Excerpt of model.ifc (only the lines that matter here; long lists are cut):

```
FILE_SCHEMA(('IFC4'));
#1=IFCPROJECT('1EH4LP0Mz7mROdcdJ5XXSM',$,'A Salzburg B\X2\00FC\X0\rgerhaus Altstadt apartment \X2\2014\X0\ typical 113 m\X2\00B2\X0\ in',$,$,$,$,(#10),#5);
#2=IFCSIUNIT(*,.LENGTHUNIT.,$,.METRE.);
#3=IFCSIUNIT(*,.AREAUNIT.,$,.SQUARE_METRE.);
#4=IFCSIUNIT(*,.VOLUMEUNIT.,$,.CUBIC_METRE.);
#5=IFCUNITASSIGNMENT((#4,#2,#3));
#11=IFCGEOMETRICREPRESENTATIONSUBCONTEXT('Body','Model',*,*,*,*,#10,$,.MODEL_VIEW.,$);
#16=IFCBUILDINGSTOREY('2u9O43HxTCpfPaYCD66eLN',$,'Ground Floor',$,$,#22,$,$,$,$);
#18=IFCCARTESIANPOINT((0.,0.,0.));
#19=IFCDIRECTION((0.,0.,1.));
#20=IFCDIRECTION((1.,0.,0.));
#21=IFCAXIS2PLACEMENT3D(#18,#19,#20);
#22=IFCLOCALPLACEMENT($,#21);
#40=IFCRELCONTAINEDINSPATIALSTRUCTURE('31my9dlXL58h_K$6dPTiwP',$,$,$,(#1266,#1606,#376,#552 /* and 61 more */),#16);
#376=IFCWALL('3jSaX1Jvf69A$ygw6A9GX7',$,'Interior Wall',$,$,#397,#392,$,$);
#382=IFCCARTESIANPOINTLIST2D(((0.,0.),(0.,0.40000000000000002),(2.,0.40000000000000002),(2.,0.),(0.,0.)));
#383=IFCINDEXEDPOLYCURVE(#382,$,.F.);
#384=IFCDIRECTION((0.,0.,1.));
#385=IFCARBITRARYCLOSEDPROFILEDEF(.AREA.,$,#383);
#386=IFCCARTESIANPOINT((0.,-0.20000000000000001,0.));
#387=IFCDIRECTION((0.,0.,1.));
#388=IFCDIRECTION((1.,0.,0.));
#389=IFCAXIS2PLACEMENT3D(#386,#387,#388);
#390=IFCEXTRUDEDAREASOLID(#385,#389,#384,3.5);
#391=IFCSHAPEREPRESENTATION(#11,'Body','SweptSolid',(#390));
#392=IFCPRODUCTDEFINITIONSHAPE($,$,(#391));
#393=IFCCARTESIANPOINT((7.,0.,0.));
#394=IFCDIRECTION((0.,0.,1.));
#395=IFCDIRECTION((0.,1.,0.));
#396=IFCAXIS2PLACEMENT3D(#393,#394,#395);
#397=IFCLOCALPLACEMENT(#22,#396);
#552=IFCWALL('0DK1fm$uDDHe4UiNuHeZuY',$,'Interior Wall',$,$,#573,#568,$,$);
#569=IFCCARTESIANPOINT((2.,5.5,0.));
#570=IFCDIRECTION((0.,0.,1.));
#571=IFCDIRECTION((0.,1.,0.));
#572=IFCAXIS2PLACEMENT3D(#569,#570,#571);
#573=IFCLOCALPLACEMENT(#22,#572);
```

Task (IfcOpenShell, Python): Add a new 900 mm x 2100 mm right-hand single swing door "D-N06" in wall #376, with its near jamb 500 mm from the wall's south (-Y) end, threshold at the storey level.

```python
import numpy as np
import ifcopenshell
import ifcopenshell.api.feature
import ifcopenshell.api.geometry
import ifcopenshell.api.root
import ifcopenshell.api.spatial
import ifcopenshell.geom
import ifcopenshell.util.element
import ifcopenshell.util.placement
import ifcopenshell.util.representation
import ifcopenshell.util.shape
import ifcopenshell.util.unit

model = ifcopenshell.open("model.ifc")
unit_scale = ifcopenshell.util.unit.calculate_unit_scale(model)
settings = ifcopenshell.geom.settings()


def volume(element):
    """Net volume in cubic metres, openings subtracted."""
    shape = ifcopenshell.geom.create_shape(settings, element)
    return ifcopenshell.util.shape.get_volume(shape.geometry)


wall = model.by_id(376)
storey = ifcopenshell.util.element.get_container(wall, ifc_class="IfcBuildingStorey")
context = ifcopenshell.util.representation.get_context(model, "Model", "Body", "MODEL_VIEW")
before = volume(wall)

width, height, from_end, sill = 0.9, 2.1, 0.5, 0.0  # metres

# The wall runs along its own X axis, and the end named is its -X end.
wall_shape = ifcopenshell.geom.create_shape(settings, wall)
x, y, z = ifcopenshell.util.shape.get_vertices(wall_shape.geometry).T
start = x.min() + from_end
face, thickness = float(y.min()), float(y.max() - y.min())
wall_matrix = ifcopenshell.util.placement.get_local_placement(wall.ObjectPlacement)
level = ifcopenshell.util.placement.get_local_placement(storey.ObjectPlacement)[2, 3]


def in_wall(x, y):
    """Placement at x, y metres in the wall's axes, at sill height."""
    matrix = wall_matrix.copy()
    matrix[:, 3] = wall_matrix @ np.array([x / unit_scale, y / unit_scale, 0.0, 1.0])
    matrix[2, 3] = level + sill / unit_scale
    return matrix


# Opening: a box that overshoots both wall faces by 50 mm.
opening = ifcopenshell.api.root.create_entity(model, ifc_class="IfcOpeningElement", predefined_type="OPENING")
box = ifcopenshell.api.geometry.add_wall_representation(
    model, context=context, length=width, height=height, thickness=thickness + 0.1
)
ifcopenshell.api.geometry.assign_representation(model, product=opening, representation=box)
ifcopenshell.api.geometry.edit_object_placement(model, product=opening, matrix=in_wall(start, face - 0.05), is_si=False)
ifcopenshell.api.feature.add_feature(model, feature=opening, element=wall)

door = ifcopenshell.api.root.create_entity(model, ifc_class="IfcDoor", name="D-N06", predefined_type="DOOR")
door.OverallWidth, door.OverallHeight = width / unit_scale, height / unit_scale
door.OperationType = "SINGLE_SWING_RIGHT"
body = ifcopenshell.api.geometry.add_door_representation(
    model,
    context=context,
    overall_width=door.OverallWidth,
    overall_height=door.OverallHeight,
    operation_type="SINGLE_SWING_RIGHT",
    lining_properties={"LiningDepth": thickness / unit_scale, "ThresholdDepth": thickness / unit_scale},
)
ifcopenshell.api.geometry.assign_representation(model, product=door, representation=body)
ifcopenshell.api.spatial.assign_container(model, products=[door], relating_structure=storey)
ifcopenshell.api.feature.add_filling(model, opening=opening, element=door)

# The lining spans the wall, so the door starts at the wall face.
ifcopenshell.api.geometry.edit_object_placement(model, product=door, matrix=in_wall(start, face), is_si=False)

after = volume(wall)

print(f"wall volume {before:.3f} -> {after:.3f} m3")

model.write("model_v2.ifc")
```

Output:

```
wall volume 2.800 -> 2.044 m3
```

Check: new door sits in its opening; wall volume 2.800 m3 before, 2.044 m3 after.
